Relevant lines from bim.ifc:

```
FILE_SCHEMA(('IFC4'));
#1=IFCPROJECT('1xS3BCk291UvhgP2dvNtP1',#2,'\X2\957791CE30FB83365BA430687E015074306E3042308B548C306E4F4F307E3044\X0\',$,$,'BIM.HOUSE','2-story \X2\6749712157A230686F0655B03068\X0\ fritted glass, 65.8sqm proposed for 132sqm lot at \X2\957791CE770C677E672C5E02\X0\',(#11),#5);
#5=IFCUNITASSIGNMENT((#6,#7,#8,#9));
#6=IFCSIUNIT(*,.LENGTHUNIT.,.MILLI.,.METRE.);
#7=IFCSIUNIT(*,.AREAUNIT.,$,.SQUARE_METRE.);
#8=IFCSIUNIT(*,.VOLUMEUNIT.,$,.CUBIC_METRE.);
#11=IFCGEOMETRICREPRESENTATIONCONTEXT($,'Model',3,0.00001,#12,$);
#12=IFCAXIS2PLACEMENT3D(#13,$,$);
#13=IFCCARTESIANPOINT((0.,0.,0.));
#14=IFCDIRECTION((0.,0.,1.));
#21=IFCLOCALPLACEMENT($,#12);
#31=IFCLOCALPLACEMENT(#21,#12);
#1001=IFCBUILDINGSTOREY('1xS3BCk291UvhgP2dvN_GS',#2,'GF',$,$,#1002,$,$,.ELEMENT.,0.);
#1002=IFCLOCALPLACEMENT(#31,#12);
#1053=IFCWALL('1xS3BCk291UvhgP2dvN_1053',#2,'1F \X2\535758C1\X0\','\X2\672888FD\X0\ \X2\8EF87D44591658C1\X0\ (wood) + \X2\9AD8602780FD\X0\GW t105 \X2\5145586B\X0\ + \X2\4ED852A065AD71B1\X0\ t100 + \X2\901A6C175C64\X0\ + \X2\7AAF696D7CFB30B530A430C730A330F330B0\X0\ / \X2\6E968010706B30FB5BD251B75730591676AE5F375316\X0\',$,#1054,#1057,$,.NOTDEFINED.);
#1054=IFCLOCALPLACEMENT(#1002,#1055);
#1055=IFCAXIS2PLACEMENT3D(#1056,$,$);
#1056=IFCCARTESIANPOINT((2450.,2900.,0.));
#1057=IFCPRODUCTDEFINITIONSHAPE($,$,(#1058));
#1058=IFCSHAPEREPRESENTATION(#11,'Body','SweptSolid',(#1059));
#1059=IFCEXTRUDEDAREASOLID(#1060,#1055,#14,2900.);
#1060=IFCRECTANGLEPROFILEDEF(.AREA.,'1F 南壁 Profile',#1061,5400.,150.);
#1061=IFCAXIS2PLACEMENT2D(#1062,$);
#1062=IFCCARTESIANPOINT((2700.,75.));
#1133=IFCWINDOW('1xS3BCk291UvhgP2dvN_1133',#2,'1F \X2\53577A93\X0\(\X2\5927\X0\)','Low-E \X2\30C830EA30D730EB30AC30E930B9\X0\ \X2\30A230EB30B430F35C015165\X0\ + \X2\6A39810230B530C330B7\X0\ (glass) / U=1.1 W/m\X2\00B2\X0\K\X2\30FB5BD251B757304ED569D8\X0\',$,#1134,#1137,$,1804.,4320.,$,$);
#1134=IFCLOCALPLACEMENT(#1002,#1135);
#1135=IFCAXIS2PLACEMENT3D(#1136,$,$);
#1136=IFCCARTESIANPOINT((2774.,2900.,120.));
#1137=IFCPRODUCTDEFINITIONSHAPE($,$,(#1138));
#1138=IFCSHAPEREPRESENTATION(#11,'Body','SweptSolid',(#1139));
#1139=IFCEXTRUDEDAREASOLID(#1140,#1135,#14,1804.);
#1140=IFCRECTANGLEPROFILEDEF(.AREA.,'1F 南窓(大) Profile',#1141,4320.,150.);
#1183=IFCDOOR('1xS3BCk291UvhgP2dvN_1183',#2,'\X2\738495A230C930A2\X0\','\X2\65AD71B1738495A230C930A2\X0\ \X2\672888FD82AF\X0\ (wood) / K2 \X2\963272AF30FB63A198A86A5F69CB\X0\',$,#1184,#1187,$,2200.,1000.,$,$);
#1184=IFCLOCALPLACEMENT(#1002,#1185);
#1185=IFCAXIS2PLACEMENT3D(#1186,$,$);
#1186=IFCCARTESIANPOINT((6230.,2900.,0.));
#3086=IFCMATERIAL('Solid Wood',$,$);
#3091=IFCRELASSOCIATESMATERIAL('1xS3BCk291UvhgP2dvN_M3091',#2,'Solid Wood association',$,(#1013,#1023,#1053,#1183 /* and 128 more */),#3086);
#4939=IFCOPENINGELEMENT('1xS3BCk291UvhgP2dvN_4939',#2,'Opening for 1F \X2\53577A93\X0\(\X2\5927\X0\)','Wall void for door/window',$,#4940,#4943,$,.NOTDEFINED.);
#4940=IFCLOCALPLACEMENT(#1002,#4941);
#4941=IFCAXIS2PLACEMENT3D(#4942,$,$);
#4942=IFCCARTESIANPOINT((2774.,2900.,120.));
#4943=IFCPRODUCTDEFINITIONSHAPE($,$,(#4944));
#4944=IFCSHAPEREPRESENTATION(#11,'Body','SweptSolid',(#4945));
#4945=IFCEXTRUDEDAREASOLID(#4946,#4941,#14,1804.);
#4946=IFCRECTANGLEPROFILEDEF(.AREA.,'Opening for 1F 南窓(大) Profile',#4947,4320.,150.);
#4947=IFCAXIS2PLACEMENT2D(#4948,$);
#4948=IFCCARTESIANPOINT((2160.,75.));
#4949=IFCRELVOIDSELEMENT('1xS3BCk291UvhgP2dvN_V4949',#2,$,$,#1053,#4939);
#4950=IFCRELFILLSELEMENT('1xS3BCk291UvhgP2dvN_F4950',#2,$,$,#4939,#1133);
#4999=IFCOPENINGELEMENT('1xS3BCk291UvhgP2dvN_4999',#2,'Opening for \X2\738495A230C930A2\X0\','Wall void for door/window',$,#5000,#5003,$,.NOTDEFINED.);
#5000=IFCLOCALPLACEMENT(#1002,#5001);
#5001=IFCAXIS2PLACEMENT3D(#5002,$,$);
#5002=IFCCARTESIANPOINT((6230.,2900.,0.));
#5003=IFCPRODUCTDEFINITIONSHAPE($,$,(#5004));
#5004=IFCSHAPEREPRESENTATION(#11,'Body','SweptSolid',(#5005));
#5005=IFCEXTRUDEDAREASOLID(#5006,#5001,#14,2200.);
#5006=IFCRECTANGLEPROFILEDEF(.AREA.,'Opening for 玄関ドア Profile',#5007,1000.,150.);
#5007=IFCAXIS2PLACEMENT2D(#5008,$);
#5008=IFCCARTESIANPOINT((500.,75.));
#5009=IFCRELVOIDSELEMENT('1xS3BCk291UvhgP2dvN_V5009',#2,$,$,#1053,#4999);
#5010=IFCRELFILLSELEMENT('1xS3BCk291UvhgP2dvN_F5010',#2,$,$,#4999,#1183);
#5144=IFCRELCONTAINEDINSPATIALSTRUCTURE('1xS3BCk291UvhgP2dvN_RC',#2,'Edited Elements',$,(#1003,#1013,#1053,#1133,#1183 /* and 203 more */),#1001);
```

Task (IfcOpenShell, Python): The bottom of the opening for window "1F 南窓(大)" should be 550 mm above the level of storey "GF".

```python
import numpy as np
import ifcopenshell
import ifcopenshell.api.geometry
import ifcopenshell.geom
import ifcopenshell.util.element
import ifcopenshell.util.placement
import ifcopenshell.util.shape
import ifcopenshell.util.unit

model = ifcopenshell.open("bim.ifc")
unit_scale = ifcopenshell.util.unit.calculate_unit_scale(model)

window = model.by_id(1133)
opening = window.FillsVoids[0].RelatingOpeningElement
storey = ifcopenshell.util.element.get_container(window, ifc_class="IfcBuildingStorey")
level = ifcopenshell.util.placement.get_local_placement(storey.ObjectPlacement)[2, 3]

# The opening's origin need not be at the sill, so measure its lowest point.
shape = ifcopenshell.geom.create_shape(ifcopenshell.geom.settings(), opening)
bottom = ifcopenshell.util.shape.get_shape_bottom_elevation(shape, shape.geometry) / unit_scale
dz = level + 550.0 - bottom

shift = np.array([0.0, 0.0, dz])
# The window is not placed relative to its opening, so move both.
for product in (opening, window):
    matrix = ifcopenshell.util.placement.get_local_placement(product.ObjectPlacement)
    matrix[:3, 3] += shift
    ifcopenshell.api.geometry.edit_object_placement(model, product=product, matrix=matrix, is_si=False)

print(f"moved by {dz * unit_scale:+.3f} m")

model.write("bim_edited.ifc")
```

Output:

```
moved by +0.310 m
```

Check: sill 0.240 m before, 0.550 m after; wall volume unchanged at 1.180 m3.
